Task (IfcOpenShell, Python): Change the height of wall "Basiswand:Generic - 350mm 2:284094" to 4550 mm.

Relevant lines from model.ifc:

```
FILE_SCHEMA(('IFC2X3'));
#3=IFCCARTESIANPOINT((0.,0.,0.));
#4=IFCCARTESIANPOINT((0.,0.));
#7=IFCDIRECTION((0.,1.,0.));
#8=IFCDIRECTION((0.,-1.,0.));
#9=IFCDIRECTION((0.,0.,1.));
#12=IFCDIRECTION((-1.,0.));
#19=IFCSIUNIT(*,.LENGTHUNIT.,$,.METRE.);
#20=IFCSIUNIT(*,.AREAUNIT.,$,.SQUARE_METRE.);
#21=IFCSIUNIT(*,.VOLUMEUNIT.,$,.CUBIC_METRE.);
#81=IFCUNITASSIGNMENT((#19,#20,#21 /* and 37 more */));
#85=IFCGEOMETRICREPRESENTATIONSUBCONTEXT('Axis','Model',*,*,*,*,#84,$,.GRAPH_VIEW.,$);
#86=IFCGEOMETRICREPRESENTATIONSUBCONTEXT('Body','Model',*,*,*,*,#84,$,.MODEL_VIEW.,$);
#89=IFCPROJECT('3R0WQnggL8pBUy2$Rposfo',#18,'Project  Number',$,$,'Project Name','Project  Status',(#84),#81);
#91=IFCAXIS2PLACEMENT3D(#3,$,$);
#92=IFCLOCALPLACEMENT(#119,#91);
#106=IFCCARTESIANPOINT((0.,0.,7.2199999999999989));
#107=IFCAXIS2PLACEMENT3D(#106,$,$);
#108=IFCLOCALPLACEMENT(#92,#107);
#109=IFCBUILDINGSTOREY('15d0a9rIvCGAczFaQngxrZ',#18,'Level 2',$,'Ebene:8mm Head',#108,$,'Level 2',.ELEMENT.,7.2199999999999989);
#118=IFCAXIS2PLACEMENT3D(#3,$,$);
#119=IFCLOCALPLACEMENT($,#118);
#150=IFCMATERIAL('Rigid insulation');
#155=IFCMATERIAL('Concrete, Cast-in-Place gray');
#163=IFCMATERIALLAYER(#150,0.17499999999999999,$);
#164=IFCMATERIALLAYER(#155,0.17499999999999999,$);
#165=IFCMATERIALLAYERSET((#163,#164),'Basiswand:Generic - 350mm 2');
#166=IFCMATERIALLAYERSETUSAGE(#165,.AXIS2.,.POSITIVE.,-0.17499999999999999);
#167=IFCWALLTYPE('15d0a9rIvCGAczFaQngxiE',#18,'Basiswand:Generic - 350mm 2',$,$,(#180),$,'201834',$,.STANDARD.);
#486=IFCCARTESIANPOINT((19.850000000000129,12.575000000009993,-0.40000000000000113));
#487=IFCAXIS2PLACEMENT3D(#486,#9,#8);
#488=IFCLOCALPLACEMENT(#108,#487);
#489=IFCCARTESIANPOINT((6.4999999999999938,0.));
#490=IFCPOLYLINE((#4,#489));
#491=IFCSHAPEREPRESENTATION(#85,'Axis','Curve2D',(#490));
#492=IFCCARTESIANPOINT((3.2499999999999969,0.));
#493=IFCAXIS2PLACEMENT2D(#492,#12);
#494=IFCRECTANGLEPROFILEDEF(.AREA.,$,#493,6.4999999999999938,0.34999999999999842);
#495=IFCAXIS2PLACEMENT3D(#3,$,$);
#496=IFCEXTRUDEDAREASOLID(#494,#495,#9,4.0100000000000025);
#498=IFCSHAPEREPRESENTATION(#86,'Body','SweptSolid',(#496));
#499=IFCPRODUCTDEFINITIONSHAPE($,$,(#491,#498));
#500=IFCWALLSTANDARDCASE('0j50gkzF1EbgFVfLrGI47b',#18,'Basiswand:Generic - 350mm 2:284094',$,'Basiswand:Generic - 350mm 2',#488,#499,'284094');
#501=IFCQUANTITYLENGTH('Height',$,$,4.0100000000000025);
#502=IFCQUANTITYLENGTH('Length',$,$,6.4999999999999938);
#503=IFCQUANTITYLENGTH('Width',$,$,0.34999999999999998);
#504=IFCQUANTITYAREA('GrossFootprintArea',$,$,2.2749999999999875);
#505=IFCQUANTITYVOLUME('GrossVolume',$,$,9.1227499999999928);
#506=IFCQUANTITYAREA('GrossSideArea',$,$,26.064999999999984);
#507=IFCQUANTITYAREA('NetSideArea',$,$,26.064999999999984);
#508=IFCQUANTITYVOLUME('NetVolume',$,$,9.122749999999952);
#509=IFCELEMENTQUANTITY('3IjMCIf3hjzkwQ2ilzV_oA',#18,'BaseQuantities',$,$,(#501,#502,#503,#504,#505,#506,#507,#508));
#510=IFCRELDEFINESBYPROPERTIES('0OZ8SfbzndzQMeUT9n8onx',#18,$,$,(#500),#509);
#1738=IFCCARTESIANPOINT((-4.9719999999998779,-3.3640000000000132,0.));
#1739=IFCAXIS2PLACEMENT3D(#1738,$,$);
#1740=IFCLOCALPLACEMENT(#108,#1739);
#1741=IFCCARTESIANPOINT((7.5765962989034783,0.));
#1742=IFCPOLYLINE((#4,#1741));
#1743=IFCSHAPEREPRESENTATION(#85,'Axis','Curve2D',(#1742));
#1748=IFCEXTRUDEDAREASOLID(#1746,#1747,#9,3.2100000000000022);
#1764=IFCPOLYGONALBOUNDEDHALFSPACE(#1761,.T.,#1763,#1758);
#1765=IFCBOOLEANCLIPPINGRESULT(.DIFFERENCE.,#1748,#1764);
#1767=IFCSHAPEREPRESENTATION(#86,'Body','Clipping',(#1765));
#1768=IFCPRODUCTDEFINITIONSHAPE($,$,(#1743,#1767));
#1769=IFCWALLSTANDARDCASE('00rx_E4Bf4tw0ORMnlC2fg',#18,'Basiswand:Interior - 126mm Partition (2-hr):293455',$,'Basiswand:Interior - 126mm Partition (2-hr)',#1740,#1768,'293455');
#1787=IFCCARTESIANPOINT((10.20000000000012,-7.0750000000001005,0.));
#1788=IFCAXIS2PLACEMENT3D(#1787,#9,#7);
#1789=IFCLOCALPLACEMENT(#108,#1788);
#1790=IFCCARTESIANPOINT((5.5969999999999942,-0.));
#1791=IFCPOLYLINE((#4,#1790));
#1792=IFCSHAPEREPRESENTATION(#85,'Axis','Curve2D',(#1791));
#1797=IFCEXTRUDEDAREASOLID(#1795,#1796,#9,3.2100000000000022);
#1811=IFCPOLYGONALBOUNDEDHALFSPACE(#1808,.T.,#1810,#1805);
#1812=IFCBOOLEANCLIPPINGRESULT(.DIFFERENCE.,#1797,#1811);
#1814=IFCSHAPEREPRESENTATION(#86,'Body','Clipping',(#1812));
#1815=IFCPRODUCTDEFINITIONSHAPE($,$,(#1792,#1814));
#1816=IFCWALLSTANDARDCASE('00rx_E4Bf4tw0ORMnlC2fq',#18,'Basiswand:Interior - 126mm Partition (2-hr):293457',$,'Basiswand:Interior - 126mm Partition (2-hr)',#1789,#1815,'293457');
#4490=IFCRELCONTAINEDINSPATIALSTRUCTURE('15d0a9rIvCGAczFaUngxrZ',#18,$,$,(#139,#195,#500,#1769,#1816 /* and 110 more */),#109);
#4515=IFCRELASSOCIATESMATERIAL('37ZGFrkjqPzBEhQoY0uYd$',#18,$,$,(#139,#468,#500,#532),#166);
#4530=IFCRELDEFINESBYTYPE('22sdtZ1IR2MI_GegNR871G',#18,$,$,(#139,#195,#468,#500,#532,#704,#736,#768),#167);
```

```python
import ifcopenshell
import ifcopenshell.api.pset
import ifcopenshell.geom
import ifcopenshell.util.element
import ifcopenshell.util.representation
import ifcopenshell.util.shape
import ifcopenshell.util.unit

model = ifcopenshell.open("model.ifc")
unit_scale = ifcopenshell.util.unit.calculate_unit_scale(model)
area_scale = ifcopenshell.util.unit.calculate_unit_scale(model, "AREAUNIT")
volume_scale = ifcopenshell.util.unit.calculate_unit_scale(model, "VOLUMEUNIT")
settings = ifcopenshell.geom.settings()


def volume(element):
    """Net volume in cubic metres, openings subtracted."""
    shape = ifcopenshell.geom.create_shape(settings, element)
    return ifcopenshell.util.shape.get_volume(shape.geometry)


wall = model.by_id(500)
before = volume(wall)

body = ifcopenshell.util.representation.get_representation(wall, "Model", "Body")
solid = body.Items[0]
old_height = solid.Depth
solid.Depth = 4.55
after = volume(wall)
thickness = 0.35  # wall thickness in metres

# Update the stored height, areas and volumes.
qto = model.by_id(ifcopenshell.util.element.get_pset(wall, "BaseQuantities", should_inherit=False)["id"])
ifcopenshell.api.pset.edit_qto(model, qto=qto, properties={
    "Height": solid.Depth,
    "GrossVolume": ifcopenshell.util.element.get_pset(wall, "BaseQuantities", "GrossVolume") * solid.Depth / old_height,
    "GrossSideArea": ifcopenshell.util.element.get_pset(wall, "BaseQuantities", "GrossSideArea") * solid.Depth / old_height,
    "NetSideArea": after / thickness / area_scale,
    "NetVolume": after / volume_scale,
})

print(f"height {old_height:g} -> {solid.Depth:g}, volume {before:.3f} -> {after:.3f} m3")

model.write("model_rev.ifc")
```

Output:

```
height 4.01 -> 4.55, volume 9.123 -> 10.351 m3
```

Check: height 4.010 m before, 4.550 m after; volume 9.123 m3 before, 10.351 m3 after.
